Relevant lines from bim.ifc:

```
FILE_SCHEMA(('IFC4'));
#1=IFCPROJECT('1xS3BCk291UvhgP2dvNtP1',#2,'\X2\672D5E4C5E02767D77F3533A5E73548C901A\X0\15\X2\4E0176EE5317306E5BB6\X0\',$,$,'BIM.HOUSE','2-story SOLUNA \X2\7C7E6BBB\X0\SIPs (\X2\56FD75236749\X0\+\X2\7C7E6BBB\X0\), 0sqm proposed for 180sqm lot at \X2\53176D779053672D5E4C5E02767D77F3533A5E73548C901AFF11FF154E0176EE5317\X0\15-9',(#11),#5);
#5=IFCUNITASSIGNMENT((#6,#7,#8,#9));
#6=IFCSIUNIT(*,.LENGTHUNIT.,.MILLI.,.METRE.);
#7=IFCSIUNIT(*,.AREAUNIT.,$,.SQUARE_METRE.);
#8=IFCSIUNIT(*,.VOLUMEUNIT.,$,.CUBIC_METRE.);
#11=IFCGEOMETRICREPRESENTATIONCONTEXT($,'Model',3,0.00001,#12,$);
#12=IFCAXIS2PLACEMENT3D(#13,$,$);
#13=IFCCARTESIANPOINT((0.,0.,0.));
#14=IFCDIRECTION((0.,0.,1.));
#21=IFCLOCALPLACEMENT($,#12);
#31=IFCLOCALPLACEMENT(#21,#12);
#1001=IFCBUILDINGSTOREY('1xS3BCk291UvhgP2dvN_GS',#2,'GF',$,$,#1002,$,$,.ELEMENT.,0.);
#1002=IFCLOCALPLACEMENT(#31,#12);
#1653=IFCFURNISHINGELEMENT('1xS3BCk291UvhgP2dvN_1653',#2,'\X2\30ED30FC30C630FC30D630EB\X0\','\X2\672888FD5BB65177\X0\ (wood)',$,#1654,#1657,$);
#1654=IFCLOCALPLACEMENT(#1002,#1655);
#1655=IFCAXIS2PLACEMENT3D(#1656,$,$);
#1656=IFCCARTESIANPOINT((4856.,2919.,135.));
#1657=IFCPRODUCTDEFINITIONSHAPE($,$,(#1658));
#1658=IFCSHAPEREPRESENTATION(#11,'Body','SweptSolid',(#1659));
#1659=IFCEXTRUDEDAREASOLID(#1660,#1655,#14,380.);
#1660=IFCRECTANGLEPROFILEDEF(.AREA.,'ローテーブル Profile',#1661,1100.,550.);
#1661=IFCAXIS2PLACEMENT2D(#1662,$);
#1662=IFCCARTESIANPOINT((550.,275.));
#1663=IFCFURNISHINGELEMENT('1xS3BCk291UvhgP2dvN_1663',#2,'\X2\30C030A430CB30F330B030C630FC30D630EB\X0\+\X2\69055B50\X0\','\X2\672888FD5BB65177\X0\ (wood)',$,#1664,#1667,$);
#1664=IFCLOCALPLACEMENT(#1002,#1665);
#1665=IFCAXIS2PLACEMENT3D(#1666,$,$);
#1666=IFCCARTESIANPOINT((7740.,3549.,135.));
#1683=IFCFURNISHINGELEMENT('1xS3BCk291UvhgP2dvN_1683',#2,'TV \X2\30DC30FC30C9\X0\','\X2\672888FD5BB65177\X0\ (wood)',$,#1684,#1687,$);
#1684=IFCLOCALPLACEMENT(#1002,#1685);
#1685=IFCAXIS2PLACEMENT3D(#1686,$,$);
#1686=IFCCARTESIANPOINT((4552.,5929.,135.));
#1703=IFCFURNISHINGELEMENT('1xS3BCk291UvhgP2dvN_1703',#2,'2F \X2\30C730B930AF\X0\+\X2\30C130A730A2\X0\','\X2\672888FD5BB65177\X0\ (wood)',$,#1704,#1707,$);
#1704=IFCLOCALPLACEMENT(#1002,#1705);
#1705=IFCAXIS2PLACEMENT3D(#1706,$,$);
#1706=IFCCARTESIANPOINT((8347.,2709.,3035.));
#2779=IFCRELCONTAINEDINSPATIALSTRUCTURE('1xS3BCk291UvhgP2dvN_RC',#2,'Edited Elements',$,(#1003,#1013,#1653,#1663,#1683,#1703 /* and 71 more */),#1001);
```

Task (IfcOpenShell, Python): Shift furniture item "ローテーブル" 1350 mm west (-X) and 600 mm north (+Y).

```python
import ifcopenshell
import ifcopenshell.api.geometry
import ifcopenshell.util.placement
import ifcopenshell.util.unit

model = ifcopenshell.open("bim.ifc")
unit_scale = ifcopenshell.util.unit.calculate_unit_scale(model)

item = model.by_id(1653)
matrix = ifcopenshell.util.placement.get_local_placement(item.ObjectPlacement)
matrix[0, 3] -= 1.35 / unit_scale
matrix[1, 3] += 0.6 / unit_scale
ifcopenshell.api.geometry.edit_object_placement(model, product=item, matrix=matrix, is_si=False)

print(ifcopenshell.util.placement.get_local_placement(item.ObjectPlacement).round(3) + 0.0)

model.write("bim_edited.ifc")
```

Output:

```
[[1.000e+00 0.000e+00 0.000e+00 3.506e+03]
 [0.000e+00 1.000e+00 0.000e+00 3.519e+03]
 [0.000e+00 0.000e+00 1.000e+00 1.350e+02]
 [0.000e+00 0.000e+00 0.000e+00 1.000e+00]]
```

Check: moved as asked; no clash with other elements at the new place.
